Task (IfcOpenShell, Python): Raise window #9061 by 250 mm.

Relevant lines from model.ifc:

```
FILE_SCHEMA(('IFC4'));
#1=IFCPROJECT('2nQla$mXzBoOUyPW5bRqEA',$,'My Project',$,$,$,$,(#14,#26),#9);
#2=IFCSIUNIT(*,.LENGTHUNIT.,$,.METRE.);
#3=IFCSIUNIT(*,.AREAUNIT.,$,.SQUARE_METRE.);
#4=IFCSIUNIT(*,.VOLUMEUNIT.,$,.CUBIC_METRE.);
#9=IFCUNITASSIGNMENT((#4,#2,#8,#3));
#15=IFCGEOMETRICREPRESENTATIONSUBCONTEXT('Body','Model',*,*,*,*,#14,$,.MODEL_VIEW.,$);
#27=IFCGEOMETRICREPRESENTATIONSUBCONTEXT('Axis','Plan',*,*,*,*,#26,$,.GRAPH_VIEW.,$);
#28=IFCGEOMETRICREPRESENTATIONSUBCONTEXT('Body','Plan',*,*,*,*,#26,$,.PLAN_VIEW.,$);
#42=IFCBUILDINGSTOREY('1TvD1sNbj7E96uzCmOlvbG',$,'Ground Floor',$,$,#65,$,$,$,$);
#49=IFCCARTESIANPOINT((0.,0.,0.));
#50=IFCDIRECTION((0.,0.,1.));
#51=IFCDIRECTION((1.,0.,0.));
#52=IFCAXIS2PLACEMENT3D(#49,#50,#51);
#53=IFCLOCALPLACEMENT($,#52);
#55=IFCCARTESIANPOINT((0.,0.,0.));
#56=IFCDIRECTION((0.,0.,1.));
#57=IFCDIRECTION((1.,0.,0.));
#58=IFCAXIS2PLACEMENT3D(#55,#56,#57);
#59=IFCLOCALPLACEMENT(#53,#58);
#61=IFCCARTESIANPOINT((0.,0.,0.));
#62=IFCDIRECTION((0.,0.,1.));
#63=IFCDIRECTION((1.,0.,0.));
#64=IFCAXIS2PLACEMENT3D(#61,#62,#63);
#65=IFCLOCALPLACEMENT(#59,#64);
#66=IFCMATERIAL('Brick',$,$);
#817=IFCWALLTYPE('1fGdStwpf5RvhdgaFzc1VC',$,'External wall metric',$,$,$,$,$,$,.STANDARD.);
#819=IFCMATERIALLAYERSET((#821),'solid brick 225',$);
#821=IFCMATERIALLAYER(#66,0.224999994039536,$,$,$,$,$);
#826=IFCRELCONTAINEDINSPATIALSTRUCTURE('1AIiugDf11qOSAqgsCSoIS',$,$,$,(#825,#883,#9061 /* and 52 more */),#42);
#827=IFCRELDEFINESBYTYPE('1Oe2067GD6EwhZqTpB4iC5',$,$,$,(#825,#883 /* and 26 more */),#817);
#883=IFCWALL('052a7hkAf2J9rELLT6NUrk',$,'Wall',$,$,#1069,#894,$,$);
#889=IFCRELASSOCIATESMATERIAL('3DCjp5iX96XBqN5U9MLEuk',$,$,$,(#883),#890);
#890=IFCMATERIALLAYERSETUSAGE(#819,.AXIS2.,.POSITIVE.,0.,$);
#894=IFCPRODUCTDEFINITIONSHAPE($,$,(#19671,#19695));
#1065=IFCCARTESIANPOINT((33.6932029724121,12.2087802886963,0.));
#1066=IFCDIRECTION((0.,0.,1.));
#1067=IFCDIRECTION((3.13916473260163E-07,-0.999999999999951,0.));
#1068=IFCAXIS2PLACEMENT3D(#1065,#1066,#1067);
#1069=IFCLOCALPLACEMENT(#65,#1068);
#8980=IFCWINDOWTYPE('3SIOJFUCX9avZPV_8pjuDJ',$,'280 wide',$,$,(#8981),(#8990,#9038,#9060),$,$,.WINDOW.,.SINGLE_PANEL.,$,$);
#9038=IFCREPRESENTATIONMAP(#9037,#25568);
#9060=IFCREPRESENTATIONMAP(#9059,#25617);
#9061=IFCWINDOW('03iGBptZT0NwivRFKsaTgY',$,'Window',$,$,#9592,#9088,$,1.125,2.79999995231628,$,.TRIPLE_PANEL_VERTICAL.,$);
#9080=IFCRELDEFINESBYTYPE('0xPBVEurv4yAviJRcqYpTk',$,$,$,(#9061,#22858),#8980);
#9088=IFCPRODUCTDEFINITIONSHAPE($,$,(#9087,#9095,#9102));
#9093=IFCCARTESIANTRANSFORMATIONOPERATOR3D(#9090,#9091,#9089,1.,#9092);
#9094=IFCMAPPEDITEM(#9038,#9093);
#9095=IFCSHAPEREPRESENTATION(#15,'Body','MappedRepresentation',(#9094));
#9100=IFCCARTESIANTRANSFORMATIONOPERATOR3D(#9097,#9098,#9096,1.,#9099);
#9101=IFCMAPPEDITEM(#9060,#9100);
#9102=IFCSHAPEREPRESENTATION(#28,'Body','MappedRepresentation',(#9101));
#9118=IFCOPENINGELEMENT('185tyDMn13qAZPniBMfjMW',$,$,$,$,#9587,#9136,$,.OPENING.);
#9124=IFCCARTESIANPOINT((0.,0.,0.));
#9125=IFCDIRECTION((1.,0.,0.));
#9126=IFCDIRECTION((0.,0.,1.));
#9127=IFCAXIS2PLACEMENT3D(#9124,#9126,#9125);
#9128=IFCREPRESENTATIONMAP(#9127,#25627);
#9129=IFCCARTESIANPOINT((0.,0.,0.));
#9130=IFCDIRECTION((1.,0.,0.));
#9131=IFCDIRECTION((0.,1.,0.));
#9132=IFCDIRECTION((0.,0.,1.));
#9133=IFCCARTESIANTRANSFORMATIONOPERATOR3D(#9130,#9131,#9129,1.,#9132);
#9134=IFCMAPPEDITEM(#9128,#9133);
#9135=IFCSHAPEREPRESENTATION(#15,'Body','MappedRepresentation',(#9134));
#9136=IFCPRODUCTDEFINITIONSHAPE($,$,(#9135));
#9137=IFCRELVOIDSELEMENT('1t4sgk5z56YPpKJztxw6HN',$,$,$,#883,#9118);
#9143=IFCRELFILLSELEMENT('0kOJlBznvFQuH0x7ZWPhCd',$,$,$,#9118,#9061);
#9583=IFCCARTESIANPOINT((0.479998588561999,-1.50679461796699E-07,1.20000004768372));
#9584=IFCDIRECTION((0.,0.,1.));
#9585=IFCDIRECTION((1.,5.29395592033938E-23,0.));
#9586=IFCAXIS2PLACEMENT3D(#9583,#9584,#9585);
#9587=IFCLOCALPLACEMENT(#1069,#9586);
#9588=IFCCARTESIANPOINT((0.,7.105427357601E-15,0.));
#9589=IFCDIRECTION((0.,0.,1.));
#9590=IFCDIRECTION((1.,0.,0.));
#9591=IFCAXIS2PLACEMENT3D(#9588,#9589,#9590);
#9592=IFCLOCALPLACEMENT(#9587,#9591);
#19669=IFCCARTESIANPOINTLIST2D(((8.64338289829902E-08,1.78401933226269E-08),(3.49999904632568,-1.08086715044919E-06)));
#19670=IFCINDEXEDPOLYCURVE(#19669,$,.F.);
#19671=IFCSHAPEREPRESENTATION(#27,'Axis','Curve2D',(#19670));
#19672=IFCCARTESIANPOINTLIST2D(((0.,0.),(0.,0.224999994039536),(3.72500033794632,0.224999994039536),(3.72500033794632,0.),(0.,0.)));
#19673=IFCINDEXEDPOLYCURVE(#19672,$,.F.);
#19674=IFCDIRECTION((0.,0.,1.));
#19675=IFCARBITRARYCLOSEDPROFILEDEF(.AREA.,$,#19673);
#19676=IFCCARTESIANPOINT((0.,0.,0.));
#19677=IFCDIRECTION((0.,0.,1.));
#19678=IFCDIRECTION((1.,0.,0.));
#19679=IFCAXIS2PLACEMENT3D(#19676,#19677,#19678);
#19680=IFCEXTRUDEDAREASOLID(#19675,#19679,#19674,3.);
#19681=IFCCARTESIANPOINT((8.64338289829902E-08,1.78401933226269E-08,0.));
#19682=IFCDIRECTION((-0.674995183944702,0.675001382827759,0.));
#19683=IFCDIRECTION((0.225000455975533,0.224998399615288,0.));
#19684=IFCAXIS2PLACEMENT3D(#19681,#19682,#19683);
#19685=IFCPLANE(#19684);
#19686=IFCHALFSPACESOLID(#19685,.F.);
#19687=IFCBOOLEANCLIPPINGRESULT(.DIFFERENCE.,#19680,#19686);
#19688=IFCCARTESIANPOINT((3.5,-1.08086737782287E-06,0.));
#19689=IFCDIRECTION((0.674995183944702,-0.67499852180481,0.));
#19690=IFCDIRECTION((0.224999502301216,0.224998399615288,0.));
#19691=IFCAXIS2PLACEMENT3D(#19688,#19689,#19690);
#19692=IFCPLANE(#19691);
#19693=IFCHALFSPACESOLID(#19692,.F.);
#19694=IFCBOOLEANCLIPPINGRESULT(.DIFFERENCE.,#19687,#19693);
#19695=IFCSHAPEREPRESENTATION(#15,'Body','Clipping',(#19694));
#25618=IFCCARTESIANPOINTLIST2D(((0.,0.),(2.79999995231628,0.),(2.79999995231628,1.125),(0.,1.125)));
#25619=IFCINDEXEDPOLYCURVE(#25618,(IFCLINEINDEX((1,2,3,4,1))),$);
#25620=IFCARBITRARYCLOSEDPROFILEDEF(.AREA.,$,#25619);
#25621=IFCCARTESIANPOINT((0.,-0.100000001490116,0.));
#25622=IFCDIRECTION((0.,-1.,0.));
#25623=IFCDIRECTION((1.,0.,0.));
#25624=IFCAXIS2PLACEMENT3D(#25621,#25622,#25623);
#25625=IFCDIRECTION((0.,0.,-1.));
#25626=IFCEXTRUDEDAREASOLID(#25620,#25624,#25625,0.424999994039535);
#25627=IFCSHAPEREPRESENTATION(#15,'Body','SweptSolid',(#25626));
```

```python
import numpy as np
import ifcopenshell
import ifcopenshell.api.geometry
import ifcopenshell.util.placement
import ifcopenshell.util.unit

model = ifcopenshell.open("model.ifc")
unit_scale = ifcopenshell.util.unit.calculate_unit_scale(model)

window = model.by_guid("03iGBptZT0NwivRFKsaTgY")
opening = window.FillsVoids[0].RelatingOpeningElement
dz = 0.25 / unit_scale

shift = np.array([0.0, 0.0, dz])
# The window is placed relative to its opening, so it follows when the opening moves.
matrix = ifcopenshell.util.placement.get_local_placement(opening.ObjectPlacement)
matrix[:3, 3] += shift
ifcopenshell.api.geometry.edit_object_placement(
    model, product=opening, matrix=matrix, is_si=False, should_transform_children=True
)

print(f"moved by {dz * unit_scale:+.3f} m")

model.write("model_v2.ifc")
```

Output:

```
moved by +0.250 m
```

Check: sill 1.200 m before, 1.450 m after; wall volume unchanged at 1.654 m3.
